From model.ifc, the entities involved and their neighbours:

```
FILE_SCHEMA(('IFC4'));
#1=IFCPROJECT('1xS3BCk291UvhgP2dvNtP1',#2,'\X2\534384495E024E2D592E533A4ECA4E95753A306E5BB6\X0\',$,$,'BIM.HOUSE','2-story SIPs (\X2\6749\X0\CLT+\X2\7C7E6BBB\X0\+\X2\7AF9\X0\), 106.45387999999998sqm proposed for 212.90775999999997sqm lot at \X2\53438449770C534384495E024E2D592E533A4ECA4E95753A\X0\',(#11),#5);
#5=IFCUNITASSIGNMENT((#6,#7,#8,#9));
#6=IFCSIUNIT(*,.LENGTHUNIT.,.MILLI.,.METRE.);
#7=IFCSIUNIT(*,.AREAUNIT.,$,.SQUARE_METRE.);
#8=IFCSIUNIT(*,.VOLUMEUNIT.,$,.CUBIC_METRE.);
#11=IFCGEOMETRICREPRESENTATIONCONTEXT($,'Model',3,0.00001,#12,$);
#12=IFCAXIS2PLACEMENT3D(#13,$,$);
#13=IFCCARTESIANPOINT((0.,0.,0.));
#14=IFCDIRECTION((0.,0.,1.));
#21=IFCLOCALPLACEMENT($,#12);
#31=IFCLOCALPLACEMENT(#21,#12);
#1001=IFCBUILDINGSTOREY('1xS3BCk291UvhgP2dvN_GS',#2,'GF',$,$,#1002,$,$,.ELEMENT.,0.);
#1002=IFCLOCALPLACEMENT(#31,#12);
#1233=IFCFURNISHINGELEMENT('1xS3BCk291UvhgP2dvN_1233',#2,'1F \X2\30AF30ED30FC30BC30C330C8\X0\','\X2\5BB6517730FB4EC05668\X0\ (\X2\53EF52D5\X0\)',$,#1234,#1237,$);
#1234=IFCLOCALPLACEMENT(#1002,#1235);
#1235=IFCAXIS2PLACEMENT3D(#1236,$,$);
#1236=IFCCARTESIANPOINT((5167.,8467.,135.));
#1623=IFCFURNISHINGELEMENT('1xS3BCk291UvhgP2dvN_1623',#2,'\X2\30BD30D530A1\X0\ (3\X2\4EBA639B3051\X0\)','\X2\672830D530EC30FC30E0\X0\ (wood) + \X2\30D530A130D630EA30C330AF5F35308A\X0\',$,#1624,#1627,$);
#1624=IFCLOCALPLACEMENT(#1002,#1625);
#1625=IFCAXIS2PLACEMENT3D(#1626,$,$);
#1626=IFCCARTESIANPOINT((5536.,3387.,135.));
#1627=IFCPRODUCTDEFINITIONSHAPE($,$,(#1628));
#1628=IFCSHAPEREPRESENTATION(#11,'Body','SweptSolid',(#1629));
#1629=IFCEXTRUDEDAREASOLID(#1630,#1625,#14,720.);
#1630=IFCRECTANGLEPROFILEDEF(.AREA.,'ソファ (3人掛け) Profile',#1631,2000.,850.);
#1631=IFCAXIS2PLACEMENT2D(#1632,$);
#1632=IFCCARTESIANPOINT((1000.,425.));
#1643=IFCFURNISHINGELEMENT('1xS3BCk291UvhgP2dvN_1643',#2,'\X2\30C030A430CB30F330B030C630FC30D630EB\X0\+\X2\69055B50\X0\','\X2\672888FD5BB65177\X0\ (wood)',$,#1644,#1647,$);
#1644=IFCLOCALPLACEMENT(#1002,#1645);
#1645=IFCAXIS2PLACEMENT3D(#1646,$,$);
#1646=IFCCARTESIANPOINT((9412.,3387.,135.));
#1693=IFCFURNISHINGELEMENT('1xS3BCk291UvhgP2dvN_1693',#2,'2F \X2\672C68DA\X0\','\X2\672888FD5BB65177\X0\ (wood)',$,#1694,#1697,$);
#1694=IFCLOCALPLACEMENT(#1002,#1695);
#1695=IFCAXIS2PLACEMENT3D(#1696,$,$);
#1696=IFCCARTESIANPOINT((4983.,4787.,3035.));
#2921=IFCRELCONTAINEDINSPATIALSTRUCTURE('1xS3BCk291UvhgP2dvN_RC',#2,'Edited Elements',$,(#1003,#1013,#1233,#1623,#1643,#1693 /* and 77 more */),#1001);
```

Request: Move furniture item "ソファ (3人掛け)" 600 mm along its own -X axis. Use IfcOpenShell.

```python
import ifcopenshell
import ifcopenshell.api.geometry
import ifcopenshell.util.placement

model = ifcopenshell.open("model.ifc")

item = model.by_guid("1xS3BCk291UvhgP2dvN_1623")
matrix = ifcopenshell.util.placement.get_local_placement(item.ObjectPlacement)
matrix[:3, 3] -= matrix[:3, 0] * 600.0
ifcopenshell.api.geometry.edit_object_placement(model, product=item, matrix=matrix, is_si=False)

print(ifcopenshell.util.placement.get_local_placement(item.ObjectPlacement).round(3) + 0.0)

model.write("model_v2.ifc")
```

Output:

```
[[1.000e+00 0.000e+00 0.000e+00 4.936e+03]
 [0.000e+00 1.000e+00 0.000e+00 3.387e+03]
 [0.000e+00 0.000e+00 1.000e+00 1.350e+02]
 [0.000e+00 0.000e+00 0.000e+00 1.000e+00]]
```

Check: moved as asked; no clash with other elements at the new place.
